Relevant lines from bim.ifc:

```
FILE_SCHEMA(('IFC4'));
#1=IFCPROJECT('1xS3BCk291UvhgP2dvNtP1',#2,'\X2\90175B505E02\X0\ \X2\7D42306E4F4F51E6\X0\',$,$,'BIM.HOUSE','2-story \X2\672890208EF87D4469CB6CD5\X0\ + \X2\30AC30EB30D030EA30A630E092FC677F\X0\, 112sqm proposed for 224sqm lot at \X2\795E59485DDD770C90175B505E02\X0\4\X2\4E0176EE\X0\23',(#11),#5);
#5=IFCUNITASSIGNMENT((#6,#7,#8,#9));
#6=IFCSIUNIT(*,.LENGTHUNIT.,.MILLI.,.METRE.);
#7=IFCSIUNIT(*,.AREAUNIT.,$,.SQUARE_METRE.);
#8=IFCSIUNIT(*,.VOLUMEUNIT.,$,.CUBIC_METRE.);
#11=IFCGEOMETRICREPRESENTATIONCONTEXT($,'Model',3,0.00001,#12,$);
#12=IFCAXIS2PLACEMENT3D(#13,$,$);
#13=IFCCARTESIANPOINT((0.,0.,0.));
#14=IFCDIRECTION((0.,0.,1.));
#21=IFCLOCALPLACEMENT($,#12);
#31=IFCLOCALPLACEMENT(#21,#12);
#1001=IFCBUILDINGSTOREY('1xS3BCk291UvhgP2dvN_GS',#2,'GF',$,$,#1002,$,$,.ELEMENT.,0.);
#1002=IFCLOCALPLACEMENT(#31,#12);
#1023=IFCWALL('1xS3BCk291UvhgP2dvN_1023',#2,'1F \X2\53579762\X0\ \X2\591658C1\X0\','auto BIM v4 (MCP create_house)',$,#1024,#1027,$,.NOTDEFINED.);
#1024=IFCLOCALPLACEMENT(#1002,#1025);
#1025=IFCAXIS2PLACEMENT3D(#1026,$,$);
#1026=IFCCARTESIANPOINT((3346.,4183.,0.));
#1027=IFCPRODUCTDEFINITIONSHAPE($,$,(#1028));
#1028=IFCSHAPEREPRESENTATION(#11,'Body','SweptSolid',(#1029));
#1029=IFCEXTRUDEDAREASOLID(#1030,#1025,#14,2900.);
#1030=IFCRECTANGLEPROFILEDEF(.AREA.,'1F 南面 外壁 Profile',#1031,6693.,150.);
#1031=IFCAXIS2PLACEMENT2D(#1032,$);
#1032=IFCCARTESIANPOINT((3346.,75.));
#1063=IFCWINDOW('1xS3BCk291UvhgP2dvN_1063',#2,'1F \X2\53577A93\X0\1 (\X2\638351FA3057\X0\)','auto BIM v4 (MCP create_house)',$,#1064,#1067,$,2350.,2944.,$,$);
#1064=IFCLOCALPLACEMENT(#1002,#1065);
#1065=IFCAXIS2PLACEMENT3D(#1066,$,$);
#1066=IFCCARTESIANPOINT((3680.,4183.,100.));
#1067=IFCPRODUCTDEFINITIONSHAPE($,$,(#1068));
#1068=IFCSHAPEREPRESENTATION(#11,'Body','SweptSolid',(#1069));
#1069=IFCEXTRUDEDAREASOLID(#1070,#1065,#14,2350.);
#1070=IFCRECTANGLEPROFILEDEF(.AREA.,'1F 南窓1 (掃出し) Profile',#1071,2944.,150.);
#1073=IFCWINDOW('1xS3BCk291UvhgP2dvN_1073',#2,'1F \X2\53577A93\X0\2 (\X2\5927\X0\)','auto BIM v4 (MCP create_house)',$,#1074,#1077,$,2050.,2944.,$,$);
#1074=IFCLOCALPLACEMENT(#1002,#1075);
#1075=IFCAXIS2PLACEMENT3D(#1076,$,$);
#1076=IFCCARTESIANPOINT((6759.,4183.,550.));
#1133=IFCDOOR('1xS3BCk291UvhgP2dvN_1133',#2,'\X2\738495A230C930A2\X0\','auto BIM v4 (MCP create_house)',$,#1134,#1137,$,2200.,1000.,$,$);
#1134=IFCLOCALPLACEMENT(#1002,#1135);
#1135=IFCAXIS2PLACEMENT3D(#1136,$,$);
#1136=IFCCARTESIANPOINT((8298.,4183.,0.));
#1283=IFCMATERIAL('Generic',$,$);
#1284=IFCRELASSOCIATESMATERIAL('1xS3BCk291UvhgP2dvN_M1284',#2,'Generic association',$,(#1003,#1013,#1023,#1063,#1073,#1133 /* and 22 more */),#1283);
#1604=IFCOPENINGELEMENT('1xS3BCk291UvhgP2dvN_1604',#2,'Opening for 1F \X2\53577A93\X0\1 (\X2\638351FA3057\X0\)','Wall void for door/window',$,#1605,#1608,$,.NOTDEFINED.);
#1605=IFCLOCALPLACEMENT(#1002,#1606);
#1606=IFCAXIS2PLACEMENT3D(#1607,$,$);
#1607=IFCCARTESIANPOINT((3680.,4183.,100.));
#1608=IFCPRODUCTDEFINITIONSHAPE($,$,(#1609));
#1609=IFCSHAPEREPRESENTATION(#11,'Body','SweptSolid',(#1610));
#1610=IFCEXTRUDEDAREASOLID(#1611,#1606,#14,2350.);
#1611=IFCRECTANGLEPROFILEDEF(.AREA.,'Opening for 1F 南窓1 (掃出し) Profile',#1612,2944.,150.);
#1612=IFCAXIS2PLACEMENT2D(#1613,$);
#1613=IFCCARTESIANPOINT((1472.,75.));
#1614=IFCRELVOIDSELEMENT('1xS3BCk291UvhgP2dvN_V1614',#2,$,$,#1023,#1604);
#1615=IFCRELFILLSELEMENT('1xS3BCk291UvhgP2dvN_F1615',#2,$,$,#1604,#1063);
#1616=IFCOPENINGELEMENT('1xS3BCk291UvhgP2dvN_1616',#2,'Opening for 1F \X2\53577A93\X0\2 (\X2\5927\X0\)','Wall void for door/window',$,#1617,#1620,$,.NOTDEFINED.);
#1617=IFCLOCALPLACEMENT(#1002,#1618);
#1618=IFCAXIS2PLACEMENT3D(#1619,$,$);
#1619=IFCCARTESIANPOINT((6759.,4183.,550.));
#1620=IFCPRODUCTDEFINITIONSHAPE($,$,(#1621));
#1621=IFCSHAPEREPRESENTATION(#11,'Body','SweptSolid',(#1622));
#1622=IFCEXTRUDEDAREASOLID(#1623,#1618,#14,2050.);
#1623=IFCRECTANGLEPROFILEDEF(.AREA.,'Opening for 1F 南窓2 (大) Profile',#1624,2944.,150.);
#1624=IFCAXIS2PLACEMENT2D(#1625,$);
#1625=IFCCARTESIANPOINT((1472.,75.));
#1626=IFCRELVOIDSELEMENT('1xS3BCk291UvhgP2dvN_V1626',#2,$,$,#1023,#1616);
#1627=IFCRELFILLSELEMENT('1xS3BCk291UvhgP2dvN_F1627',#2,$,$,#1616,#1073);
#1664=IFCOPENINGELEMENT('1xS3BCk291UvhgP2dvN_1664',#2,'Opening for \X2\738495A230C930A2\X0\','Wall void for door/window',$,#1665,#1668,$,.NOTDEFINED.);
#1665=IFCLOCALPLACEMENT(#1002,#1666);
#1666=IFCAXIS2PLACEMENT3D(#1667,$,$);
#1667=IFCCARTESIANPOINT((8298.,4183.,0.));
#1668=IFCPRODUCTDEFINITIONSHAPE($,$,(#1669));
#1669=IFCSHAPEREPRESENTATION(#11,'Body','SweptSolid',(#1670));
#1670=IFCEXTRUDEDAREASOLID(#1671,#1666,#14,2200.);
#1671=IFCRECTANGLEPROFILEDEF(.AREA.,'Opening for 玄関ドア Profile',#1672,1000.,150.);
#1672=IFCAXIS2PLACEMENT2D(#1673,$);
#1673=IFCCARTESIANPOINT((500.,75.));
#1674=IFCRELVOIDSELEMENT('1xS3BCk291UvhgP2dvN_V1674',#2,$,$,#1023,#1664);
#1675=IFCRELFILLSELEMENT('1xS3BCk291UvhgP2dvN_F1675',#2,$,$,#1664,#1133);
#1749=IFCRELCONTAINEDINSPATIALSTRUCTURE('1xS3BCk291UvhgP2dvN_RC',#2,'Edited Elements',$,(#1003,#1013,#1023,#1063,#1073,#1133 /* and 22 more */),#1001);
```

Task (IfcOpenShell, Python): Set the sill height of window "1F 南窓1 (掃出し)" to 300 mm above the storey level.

```python
import numpy as np
import ifcopenshell
import ifcopenshell.api.geometry
import ifcopenshell.geom
import ifcopenshell.util.element
import ifcopenshell.util.placement
import ifcopenshell.util.shape
import ifcopenshell.util.unit

model = ifcopenshell.open("bim.ifc")
unit_scale = ifcopenshell.util.unit.calculate_unit_scale(model)

window = model.by_guid("1xS3BCk291UvhgP2dvN_1063")
opening = window.FillsVoids[0].RelatingOpeningElement
storey = ifcopenshell.util.element.get_container(window, ifc_class="IfcBuildingStorey")
level = ifcopenshell.util.placement.get_local_placement(storey.ObjectPlacement)[2, 3]

# The opening's origin need not be at the sill, so measure its lowest point.
shape = ifcopenshell.geom.create_shape(ifcopenshell.geom.settings(), opening)
bottom = ifcopenshell.util.shape.get_shape_bottom_elevation(shape, shape.geometry) / unit_scale
dz = level + 300.0 - bottom

shift = np.array([0.0, 0.0, dz])
# The window is not placed relative to its opening, so move both.
for product in (opening, window):
    matrix = ifcopenshell.util.placement.get_local_placement(product.ObjectPlacement)
    matrix[:3, 3] += shift
    ifcopenshell.api.geometry.edit_object_placement(model, product=product, matrix=matrix, is_si=False)

print(f"moved by {dz * unit_scale:+.3f} m")

model.write("bim_updated.ifc")
```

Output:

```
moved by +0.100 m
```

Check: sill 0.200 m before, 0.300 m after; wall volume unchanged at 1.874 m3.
